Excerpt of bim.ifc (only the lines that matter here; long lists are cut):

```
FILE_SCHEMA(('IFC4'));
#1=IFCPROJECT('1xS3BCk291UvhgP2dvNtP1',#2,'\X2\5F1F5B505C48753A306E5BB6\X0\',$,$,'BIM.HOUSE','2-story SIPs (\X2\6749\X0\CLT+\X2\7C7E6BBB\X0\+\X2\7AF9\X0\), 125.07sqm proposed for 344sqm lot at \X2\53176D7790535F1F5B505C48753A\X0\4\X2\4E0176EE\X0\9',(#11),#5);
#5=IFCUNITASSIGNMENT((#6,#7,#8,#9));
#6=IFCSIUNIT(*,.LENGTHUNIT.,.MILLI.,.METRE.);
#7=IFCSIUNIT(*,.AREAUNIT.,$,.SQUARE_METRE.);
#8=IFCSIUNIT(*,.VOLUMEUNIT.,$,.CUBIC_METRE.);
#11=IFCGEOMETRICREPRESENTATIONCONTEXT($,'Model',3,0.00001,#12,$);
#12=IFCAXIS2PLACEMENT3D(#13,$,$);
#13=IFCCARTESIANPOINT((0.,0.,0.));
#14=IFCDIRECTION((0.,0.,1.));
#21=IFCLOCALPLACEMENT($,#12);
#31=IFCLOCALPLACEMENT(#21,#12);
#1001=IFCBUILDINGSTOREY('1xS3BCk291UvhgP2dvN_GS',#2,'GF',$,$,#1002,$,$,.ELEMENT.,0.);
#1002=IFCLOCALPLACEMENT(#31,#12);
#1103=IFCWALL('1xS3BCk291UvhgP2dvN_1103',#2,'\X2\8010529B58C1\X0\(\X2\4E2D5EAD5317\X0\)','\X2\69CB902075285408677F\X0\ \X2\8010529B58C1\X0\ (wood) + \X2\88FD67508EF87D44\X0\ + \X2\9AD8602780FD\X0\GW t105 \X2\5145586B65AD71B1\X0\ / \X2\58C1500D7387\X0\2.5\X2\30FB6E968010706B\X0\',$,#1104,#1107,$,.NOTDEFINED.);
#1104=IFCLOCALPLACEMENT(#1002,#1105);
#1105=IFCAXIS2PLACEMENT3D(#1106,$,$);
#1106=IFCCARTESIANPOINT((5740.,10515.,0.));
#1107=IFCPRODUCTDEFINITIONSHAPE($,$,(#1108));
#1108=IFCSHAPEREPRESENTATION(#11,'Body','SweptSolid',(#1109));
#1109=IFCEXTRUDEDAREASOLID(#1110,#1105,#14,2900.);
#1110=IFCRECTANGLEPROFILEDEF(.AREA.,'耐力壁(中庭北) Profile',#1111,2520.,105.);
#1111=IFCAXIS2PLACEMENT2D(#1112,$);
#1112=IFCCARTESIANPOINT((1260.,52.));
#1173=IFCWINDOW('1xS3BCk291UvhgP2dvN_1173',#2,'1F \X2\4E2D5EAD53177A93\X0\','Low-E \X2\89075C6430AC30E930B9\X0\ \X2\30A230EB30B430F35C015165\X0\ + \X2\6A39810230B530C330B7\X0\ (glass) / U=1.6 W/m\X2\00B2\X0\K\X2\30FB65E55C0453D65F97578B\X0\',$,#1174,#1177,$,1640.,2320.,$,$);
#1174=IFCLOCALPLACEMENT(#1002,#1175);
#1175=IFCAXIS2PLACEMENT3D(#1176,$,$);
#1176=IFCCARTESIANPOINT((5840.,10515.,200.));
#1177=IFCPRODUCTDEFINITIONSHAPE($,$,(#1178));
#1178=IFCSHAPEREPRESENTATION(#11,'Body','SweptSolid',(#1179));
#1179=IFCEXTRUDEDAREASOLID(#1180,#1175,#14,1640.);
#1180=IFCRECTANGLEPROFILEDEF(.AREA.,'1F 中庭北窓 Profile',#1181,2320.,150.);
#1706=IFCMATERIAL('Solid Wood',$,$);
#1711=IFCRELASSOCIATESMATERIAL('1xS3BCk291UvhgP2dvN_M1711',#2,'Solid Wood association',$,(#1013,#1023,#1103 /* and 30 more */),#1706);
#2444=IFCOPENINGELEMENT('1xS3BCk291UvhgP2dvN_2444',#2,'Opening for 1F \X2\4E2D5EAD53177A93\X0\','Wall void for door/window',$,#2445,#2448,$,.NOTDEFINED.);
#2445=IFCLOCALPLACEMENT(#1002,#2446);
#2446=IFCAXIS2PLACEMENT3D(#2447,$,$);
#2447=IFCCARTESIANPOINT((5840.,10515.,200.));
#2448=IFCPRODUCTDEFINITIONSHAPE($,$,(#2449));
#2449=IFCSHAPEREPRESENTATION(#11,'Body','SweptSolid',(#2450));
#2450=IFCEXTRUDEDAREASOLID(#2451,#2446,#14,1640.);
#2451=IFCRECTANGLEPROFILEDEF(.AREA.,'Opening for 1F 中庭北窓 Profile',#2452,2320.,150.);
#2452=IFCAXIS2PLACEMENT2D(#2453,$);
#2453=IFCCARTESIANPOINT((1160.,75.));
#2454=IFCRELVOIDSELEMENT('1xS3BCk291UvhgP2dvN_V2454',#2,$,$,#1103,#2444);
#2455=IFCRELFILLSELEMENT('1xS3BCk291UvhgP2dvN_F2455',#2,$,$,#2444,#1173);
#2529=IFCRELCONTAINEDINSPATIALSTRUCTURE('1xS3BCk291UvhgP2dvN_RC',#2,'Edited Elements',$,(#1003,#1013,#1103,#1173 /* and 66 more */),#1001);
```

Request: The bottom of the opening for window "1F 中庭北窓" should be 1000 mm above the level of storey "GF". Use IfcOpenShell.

```python
import numpy as np
import ifcopenshell
import ifcopenshell.api.geometry
import ifcopenshell.geom
import ifcopenshell.util.element
import ifcopenshell.util.placement
import ifcopenshell.util.shape
import ifcopenshell.util.unit

model = ifcopenshell.open("bim.ifc")
unit_scale = ifcopenshell.util.unit.calculate_unit_scale(model)

window = model.by_guid("1xS3BCk291UvhgP2dvN_1173")
opening = window.FillsVoids[0].RelatingOpeningElement
storey = ifcopenshell.util.element.get_container(window, ifc_class="IfcBuildingStorey")
level = ifcopenshell.util.placement.get_local_placement(storey.ObjectPlacement)[2, 3]

# The opening's origin need not be at the sill, so measure its lowest point.
shape = ifcopenshell.geom.create_shape(ifcopenshell.geom.settings(), opening)
bottom = ifcopenshell.util.shape.get_shape_bottom_elevation(shape, shape.geometry) / unit_scale
dz = level + 1 / unit_scale - bottom

shift = np.array([0.0, 0.0, dz])
# The window is not placed relative to its opening, so move both.
for product in (opening, window):
    matrix = ifcopenshell.util.placement.get_local_placement(product.ObjectPlacement)
    matrix[:3, 3] += shift
    ifcopenshell.api.geometry.edit_object_placement(model, product=product, matrix=matrix, is_si=False)

print(f"moved by {dz * unit_scale:+.3f} m")

model.write("bim-out.ifc")
```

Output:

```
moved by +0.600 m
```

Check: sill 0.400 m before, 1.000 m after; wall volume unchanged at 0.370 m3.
